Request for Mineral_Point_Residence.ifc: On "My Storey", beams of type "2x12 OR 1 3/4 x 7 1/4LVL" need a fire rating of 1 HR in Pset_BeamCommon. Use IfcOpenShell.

First a look at what the model holds.

```python
import ifcopenshell
import ifcopenshell.util.element

model = ifcopenshell.open("Mineral_Point_Residence.ifc")
print(model.schema)
storey = next(s for s in model.by_type("IfcBuildingStorey") if s.Name == "My Storey")
beams = [e for e in ifcopenshell.util.element.get_decomposition(storey) if e.is_a("IfcBeam")]
seen = {}
for e in beams:
    element_type = ifcopenshell.util.element.get_type(e)
    key = (element_type.Name if element_type != e and element_type else None, ifcopenshell.util.element.get_pset(e, "Pset_BeamCommon", "FireRating"))
    seen[key] = seen.get(key, 0) + 1
for (name, value), count in sorted(seen.items(), key=str):
    print(count, "x", name, "|", value)
```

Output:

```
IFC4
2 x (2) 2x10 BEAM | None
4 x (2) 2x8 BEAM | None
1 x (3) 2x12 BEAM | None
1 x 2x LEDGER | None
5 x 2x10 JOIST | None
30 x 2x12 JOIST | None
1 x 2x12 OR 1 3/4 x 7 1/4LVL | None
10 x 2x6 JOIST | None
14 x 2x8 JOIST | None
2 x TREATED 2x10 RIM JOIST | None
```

```python
import ifcopenshell
import ifcopenshell.api.pset
import ifcopenshell.util.element

model = ifcopenshell.open("Mineral_Point_Residence.ifc")

storey = next(s for s in model.by_type("IfcBuildingStorey") if s.Name == "My Storey")
beams = [e for e in ifcopenshell.util.element.get_decomposition(storey) if e.is_a("IfcBeam")]

count = 0
for e in beams:
    element_type = ifcopenshell.util.element.get_type(e)
    if element_type in (None, e) or element_type.Name != "2x12 OR 1 3/4 x 7 1/4LVL":
        continue
    # add_pset returns the element's existing set when there is one.
    pset = ifcopenshell.api.pset.add_pset(model, product=e, name="Pset_BeamCommon")
    ifcopenshell.api.pset.edit_pset(model, pset=pset, properties={"FireRating": "1 HR"})
    count += 1

print(count, "beams updated")

model.write("Mineral_Point_Residence_updated.ifc")
```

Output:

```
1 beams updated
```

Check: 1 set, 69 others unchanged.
